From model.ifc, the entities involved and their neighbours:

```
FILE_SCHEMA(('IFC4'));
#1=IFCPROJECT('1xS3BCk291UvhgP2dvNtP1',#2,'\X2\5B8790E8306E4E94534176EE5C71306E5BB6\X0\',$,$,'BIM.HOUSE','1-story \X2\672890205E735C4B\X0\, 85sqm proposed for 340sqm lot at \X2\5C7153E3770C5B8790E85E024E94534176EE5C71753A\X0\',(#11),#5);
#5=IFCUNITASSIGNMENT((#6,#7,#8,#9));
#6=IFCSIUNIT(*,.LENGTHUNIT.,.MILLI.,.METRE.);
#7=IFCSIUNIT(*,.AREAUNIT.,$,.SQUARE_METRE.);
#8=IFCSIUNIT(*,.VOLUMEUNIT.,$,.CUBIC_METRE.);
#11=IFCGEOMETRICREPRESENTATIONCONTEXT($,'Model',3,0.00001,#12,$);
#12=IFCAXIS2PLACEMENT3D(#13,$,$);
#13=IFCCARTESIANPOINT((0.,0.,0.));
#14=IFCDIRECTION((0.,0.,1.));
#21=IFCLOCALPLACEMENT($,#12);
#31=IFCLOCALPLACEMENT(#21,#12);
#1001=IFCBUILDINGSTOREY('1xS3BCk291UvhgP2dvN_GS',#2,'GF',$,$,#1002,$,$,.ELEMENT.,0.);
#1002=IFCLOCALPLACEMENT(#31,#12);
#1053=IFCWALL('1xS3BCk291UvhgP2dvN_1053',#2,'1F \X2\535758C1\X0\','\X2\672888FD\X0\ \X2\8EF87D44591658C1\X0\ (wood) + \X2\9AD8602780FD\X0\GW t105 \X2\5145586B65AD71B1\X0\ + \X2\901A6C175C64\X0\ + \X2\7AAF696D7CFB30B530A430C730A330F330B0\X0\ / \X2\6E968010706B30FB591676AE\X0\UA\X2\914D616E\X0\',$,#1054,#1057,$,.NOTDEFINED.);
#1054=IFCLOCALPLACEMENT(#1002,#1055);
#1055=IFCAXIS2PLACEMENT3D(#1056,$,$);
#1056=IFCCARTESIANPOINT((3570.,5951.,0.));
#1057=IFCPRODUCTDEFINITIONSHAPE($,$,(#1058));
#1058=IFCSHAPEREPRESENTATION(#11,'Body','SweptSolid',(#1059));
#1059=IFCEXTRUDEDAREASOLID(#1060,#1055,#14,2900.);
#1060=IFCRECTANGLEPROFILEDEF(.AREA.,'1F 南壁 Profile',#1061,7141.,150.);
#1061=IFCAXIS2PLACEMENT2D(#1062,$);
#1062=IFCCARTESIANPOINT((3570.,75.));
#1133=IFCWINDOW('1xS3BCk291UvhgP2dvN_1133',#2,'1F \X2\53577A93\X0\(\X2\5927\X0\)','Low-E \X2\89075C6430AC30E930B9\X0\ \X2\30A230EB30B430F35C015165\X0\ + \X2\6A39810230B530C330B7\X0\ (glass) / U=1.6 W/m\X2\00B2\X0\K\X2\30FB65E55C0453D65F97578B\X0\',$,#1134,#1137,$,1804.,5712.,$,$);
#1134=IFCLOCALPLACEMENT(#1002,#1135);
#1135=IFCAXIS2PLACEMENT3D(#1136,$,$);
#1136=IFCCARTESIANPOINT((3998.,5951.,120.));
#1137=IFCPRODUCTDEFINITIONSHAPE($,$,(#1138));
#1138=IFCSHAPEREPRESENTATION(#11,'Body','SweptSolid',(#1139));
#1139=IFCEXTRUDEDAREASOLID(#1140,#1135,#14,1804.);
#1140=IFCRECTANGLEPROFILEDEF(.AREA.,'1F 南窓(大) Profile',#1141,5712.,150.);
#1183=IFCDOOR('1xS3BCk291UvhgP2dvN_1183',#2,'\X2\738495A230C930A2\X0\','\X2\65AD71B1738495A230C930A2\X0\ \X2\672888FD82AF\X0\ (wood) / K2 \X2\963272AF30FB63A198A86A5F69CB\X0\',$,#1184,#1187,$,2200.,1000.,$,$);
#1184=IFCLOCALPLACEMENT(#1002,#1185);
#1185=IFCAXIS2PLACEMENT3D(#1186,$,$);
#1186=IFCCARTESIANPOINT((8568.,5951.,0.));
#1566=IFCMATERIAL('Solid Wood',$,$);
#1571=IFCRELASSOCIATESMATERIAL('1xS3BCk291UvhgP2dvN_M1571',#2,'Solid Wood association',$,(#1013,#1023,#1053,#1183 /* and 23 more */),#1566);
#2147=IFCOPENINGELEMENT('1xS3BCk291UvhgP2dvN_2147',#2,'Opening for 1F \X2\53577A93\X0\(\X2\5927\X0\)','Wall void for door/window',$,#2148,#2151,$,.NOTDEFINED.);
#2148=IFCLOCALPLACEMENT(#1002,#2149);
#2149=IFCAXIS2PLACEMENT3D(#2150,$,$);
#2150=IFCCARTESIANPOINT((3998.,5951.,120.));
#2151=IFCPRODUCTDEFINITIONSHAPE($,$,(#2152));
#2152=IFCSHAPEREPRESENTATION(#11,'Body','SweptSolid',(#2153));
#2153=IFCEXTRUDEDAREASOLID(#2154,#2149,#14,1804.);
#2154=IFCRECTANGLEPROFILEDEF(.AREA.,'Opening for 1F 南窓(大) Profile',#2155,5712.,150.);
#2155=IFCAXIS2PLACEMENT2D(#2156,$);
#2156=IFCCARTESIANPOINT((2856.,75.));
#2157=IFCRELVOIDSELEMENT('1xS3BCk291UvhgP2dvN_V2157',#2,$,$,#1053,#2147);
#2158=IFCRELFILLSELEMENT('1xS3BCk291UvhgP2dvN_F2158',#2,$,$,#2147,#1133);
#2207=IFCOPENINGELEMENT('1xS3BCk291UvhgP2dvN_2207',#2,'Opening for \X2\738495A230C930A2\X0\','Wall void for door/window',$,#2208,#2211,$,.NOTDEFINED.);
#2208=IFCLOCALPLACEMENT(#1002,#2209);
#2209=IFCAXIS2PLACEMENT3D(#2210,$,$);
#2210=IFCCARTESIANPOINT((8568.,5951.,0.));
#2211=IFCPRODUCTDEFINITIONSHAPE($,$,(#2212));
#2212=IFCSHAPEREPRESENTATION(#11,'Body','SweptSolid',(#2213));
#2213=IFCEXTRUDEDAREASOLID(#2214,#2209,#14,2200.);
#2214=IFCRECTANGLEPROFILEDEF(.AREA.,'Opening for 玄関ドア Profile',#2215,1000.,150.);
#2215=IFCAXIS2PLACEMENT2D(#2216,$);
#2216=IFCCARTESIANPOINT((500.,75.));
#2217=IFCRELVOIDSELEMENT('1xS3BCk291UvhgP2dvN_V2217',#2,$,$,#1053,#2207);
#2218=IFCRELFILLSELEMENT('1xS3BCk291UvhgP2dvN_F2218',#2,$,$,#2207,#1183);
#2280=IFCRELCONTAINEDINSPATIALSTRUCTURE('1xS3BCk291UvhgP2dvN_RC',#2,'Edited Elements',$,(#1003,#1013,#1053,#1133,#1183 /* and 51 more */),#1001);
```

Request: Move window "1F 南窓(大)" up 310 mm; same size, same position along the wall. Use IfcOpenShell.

```python
import numpy as np
import ifcopenshell
import ifcopenshell.api.geometry
import ifcopenshell.util.placement
import ifcopenshell.util.unit

model = ifcopenshell.open("model.ifc")
unit_scale = ifcopenshell.util.unit.calculate_unit_scale(model)

window = model.by_id(1133)
opening = window.FillsVoids[0].RelatingOpeningElement
dz = 310.0

shift = np.array([0.0, 0.0, dz])
# The window is not placed relative to its opening, so move both.
for product in (opening, window):
    matrix = ifcopenshell.util.placement.get_local_placement(product.ObjectPlacement)
    matrix[:3, 3] += shift
    ifcopenshell.api.geometry.edit_object_placement(model, product=product, matrix=matrix, is_si=False)

print(f"moved by {dz * unit_scale:+.3f} m")

model.write("model-out.ifc")
```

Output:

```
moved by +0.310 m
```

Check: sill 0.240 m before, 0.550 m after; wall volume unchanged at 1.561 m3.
